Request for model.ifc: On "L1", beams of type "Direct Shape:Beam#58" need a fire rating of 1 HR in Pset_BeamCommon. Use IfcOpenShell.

First a look at what the model holds.

```python
import ifcopenshell
import ifcopenshell.util.element

model = ifcopenshell.open("model.ifc")
print(model.schema)
storey = next(s for s in model.by_type("IfcBuildingStorey") if s.Name == "L1")
beams = [e for e in ifcopenshell.util.element.get_decomposition(storey) if e.is_a("IfcBeam")]
seen = {}
for e in beams:
    element_type = ifcopenshell.util.element.get_type(e)
    key = (element_type.Name if element_type != e and element_type else None, ifcopenshell.util.element.get_pset(e, "Pset_BeamCommon", "FireRating"))
    seen[key] = seen.get(key, 0) + 1
for (name, value), count in sorted(seen.items(), key=str):
    print(count, "x", name, "|", value)
```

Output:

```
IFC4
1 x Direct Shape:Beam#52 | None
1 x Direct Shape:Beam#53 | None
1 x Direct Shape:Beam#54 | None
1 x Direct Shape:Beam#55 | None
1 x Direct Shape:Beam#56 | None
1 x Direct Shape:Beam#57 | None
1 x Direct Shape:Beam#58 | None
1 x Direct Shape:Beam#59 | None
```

```python
import ifcopenshell
import ifcopenshell.api.pset
import ifcopenshell.util.element

model = ifcopenshell.open("model.ifc")

storey = next(s for s in model.by_type("IfcBuildingStorey") if s.Name == "L1")
beams = [e for e in ifcopenshell.util.element.get_decomposition(storey) if e.is_a("IfcBeam")]

count = 0
for e in beams:
    element_type = ifcopenshell.util.element.get_type(e)
    if element_type in (None, e) or element_type.Name != "Direct Shape:Beam#58":
        continue
    # add_pset returns the element's existing set when there is one.
    pset = ifcopenshell.api.pset.add_pset(model, product=e, name="Pset_BeamCommon")
    ifcopenshell.api.pset.edit_pset(model, pset=pset, properties={"FireRating": "1 HR"})
    count += 1

print(count, "beams updated")

model.write("model_rev.ifc")
```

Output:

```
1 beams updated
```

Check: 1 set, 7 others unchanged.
